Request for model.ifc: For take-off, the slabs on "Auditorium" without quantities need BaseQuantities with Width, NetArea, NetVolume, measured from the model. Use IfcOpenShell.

First a look at what the model holds.

```python
import ifcopenshell
import ifcopenshell.util.element
import ifcopenshell.util.unit

model = ifcopenshell.open("model.ifc")
print(model.schema)
for unit_type in ("LENGTHUNIT", "AREAUNIT", "VOLUMEUNIT"):
    print(unit_type, ifcopenshell.util.unit.calculate_unit_scale(model, unit_type))
storey = next(s for s in model.by_type("IfcBuildingStorey") if s.Name == "Auditorium")
slabs = [e for e in ifcopenshell.util.element.get_decomposition(storey) if e.is_a("IfcSlab")]
for e in sorted(slabs, key=lambda e: e.id()):
    print(e.id(), e.is_a(), e.Name, list(ifcopenshell.util.element.get_psets(e, qtos_only=True)), sep=" | ")
```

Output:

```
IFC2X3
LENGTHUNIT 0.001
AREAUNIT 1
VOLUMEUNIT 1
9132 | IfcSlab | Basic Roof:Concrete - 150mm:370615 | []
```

```python
import ifcopenshell
import ifcopenshell.api.pset
import ifcopenshell.geom
import ifcopenshell.util.element
import ifcopenshell.util.shape
import ifcopenshell.util.unit

model = ifcopenshell.open("model.ifc")
unit_scale = ifcopenshell.util.unit.calculate_unit_scale(model)
area_scale = ifcopenshell.util.unit.calculate_unit_scale(model, "AREAUNIT")
volume_scale = ifcopenshell.util.unit.calculate_unit_scale(model, "VOLUMEUNIT")
settings = ifcopenshell.geom.settings()

storey = next(s for s in model.by_type("IfcBuildingStorey") if s.Name == "Auditorium")
slabs = [e for e in ifcopenshell.util.element.get_decomposition(storey) if e.is_a("IfcSlab")]

for e in sorted(slabs, key=lambda e: e.id()):
    if ifcopenshell.util.element.get_psets(e, qtos_only=True, should_inherit=False):
        continue
    # Geometry comes back in metres, in the element's own axes.
    shape = ifcopenshell.geom.create_shape(settings, e)
    values = {
        "Width": ifcopenshell.util.shape.get_z(shape.geometry) / unit_scale,
        "NetArea": ifcopenshell.util.shape.get_footprint_area(shape.geometry) / area_scale,
        "NetVolume": ifcopenshell.util.shape.get_volume(shape.geometry) / volume_scale,
    }
    qto = ifcopenshell.api.pset.add_qto(model, product=e, name="BaseQuantities")
    ifcopenshell.api.pset.edit_qto(model, qto=qto, properties=values)
    print(e.id(), {k: round(v, 3) for k, v in values.items()})

model.write("model_v2.ifc")
```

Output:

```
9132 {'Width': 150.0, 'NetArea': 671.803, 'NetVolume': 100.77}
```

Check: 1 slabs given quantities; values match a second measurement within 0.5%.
